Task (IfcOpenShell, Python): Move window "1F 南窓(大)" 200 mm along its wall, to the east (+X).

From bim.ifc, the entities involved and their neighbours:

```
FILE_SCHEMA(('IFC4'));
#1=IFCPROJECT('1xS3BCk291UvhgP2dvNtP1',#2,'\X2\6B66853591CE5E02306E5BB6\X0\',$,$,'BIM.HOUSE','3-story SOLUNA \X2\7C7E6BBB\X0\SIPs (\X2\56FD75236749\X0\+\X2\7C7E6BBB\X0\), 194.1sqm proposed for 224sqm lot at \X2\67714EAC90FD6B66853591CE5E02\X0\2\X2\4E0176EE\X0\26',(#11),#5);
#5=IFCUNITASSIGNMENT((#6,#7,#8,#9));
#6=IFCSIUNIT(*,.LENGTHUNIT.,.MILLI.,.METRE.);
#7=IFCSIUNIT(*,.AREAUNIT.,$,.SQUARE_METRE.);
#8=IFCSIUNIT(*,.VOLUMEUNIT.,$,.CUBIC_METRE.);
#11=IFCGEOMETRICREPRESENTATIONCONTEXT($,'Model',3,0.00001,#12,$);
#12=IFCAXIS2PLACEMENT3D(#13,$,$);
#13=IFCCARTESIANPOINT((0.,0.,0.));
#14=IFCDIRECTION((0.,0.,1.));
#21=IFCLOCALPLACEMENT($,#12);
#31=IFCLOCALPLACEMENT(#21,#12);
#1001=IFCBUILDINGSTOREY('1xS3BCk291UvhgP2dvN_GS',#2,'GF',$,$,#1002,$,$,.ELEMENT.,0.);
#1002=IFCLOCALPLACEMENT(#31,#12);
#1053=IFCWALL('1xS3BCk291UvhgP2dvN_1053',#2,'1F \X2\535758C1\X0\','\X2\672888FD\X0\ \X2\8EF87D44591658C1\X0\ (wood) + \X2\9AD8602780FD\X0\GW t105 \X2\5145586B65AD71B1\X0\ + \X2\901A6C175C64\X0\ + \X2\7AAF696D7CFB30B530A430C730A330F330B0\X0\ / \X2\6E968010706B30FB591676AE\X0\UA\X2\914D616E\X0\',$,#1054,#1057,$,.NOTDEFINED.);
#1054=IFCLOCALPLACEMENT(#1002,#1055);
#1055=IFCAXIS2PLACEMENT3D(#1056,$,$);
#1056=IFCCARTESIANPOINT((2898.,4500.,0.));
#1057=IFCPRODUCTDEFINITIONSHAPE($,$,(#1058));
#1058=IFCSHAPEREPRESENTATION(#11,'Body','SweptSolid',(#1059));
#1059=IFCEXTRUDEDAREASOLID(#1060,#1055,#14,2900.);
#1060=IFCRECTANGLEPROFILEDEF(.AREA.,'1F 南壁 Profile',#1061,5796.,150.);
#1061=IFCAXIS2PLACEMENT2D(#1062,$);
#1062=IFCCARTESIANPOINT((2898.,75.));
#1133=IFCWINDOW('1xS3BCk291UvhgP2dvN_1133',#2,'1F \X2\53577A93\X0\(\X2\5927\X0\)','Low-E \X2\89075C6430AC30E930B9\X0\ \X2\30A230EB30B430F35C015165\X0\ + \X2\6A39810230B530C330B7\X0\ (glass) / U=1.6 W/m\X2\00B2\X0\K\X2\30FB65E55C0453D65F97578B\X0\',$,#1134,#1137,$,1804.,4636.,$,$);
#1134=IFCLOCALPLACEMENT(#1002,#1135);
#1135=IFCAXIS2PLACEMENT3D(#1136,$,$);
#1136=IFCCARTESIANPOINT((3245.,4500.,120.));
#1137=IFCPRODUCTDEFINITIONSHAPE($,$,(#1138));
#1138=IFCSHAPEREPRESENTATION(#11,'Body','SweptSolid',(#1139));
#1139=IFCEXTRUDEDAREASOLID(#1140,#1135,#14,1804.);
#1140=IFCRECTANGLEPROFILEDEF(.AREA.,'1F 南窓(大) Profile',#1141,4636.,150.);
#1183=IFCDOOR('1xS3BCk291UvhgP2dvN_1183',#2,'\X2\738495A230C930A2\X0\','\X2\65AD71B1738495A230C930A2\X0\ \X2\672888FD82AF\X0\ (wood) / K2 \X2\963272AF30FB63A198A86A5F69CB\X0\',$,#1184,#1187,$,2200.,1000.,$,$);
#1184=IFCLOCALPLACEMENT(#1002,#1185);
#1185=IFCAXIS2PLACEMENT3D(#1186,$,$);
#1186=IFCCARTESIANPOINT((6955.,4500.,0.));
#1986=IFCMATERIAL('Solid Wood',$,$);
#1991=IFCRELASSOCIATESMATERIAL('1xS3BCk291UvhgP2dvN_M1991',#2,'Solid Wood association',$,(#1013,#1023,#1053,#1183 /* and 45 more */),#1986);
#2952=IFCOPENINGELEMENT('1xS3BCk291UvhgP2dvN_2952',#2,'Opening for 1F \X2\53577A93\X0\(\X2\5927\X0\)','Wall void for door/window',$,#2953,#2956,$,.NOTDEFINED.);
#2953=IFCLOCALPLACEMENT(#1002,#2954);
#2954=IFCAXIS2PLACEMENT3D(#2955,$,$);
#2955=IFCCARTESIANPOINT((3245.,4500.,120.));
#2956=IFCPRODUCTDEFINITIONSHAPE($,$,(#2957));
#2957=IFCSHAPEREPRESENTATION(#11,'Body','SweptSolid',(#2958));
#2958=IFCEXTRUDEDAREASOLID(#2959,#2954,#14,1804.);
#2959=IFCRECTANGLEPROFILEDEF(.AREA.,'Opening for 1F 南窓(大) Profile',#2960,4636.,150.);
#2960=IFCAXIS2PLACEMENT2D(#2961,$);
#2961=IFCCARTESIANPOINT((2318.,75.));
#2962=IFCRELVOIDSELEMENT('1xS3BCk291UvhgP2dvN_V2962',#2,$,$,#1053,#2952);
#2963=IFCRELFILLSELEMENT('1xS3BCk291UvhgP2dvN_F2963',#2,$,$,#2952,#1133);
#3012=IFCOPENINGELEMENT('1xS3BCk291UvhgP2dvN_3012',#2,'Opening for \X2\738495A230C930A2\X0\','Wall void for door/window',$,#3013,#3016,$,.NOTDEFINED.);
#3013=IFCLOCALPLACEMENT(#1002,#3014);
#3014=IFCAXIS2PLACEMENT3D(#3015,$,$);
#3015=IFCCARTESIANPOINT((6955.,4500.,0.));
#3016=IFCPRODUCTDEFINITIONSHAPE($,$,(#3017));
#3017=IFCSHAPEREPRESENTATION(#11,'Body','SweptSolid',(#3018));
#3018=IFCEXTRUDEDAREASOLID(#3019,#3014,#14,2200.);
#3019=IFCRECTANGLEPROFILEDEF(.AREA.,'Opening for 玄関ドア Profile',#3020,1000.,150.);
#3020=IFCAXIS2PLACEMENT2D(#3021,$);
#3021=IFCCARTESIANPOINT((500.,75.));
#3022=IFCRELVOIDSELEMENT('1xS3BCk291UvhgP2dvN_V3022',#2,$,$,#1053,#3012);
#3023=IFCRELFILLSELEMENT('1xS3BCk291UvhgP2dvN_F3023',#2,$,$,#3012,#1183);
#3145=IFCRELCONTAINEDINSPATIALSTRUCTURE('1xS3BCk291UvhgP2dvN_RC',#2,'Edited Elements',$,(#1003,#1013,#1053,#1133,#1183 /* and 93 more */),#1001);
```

```python
import ifcopenshell
import ifcopenshell.api.geometry
import ifcopenshell.util.placement
import ifcopenshell.util.unit

model = ifcopenshell.open("bim.ifc")
unit_scale = ifcopenshell.util.unit.calculate_unit_scale(model)

window = model.by_guid("1xS3BCk291UvhgP2dvN_1133")
opening = window.FillsVoids[0].RelatingOpeningElement
wall = opening.VoidsElements[0].RelatingBuildingElement

wall_matrix = ifcopenshell.util.placement.get_local_placement(wall.ObjectPlacement)
shift = wall_matrix[:3, 0] * 0.2 / unit_scale
before = ifcopenshell.util.placement.get_local_placement(window.ObjectPlacement)[:3, 3].copy()

# The window is not placed relative to its opening, so move both.
for product in (opening, window):
    matrix = ifcopenshell.util.placement.get_local_placement(product.ObjectPlacement)
    matrix[:3, 3] += shift
    ifcopenshell.api.geometry.edit_object_placement(model, product=product, matrix=matrix, is_si=False)

after = ifcopenshell.util.placement.get_local_placement(window.ObjectPlacement)[:3, 3]
print("window moved by", (after - before).round(3) + 0.0)

model.write("bim_edited.ifc")
```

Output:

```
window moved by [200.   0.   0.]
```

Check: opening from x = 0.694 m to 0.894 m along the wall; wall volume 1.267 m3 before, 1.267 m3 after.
